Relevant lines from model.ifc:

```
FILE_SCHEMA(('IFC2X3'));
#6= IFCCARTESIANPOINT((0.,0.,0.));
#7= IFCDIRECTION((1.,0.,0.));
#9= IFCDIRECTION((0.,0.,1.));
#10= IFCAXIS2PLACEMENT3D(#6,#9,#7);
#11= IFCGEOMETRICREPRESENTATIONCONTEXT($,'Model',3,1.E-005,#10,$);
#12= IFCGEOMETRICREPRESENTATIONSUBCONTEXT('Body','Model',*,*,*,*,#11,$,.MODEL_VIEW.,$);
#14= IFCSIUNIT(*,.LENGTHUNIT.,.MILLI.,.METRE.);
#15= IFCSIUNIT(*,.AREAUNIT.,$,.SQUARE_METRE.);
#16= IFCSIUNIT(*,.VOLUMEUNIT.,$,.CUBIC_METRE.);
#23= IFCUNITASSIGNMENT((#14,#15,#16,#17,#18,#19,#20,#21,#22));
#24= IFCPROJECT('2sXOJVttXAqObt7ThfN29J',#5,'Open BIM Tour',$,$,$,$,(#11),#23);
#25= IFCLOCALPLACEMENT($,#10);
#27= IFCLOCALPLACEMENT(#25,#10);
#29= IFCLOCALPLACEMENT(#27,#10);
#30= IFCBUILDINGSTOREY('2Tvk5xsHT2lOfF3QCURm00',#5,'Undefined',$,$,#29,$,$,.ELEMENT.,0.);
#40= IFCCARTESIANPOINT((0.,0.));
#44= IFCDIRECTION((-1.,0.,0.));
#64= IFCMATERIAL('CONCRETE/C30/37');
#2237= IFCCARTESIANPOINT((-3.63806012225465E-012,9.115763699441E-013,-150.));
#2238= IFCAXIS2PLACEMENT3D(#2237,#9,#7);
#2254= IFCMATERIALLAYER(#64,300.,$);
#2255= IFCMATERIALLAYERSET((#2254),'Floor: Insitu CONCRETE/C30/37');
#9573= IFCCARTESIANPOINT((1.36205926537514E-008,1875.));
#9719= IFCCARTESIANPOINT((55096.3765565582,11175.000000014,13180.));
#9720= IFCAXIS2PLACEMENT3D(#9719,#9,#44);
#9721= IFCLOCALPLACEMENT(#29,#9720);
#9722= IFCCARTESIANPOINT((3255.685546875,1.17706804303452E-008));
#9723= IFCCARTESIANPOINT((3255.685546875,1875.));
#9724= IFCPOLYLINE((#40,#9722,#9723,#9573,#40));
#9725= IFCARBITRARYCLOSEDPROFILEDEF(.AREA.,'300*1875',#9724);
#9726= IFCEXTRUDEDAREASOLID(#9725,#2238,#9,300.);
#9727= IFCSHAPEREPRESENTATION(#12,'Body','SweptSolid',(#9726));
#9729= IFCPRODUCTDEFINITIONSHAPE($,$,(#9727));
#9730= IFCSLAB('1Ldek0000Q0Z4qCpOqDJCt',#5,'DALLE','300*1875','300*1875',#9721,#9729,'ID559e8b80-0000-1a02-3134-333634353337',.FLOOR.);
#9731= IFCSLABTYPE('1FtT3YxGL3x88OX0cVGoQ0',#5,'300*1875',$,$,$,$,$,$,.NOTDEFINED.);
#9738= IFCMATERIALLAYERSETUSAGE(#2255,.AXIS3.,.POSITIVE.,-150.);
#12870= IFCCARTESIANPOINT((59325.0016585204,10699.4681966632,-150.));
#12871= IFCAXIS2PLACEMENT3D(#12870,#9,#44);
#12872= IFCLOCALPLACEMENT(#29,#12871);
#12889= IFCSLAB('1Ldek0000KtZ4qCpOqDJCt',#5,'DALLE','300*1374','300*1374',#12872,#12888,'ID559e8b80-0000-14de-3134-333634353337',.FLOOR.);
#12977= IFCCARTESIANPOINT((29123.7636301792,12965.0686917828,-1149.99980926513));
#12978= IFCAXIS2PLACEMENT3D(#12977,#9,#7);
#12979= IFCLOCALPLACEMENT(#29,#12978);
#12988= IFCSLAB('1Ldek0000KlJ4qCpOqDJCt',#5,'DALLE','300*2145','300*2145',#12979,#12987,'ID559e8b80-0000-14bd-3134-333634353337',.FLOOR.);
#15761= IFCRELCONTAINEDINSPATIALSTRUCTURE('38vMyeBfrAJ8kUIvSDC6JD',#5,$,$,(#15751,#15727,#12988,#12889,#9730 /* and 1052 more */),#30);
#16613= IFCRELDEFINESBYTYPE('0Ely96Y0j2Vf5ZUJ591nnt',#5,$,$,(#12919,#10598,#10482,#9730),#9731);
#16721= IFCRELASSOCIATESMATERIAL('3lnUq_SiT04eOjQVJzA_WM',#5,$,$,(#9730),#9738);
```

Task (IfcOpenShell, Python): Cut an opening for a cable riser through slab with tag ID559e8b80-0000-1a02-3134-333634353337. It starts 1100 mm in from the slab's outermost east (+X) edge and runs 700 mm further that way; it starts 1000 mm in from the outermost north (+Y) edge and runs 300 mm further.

```python
import numpy as np
import ifcopenshell
import ifcopenshell.api.feature
import ifcopenshell.api.geometry
import ifcopenshell.api.root
import ifcopenshell.geom
import ifcopenshell.util.placement
import ifcopenshell.util.representation
import ifcopenshell.util.shape
import ifcopenshell.util.unit

model = ifcopenshell.open("model.ifc")
unit_scale = ifcopenshell.util.unit.calculate_unit_scale(model)
settings = ifcopenshell.geom.settings()


def volume(element):
    """Net volume in cubic metres, openings subtracted."""
    shape = ifcopenshell.geom.create_shape(settings, element)
    return ifcopenshell.util.shape.get_volume(shape.geometry)


slab = model.by_id(9730)
before = volume(slab)

# Extent in the slab's own axes, in metres. The edges named are its -X and -Y sides.
slab_shape = ifcopenshell.geom.create_shape(settings, slab)
vertices = ifcopenshell.util.shape.get_vertices(slab_shape.geometry)
x_min, y_min, bottom = vertices.min(axis=0)
top = vertices[:, 2].max()

opening = ifcopenshell.api.root.create_entity(model, ifc_class="IfcOpeningElement", name="Cable riser opening")
context = ifcopenshell.util.representation.get_context(model, "Model", "Body", "MODEL_VIEW")
width, depth = 0.7, 0.3
outline = [(0.0, 0.0), (width, 0.0), (width, depth), (0.0, depth), (0.0, 0.0)]
# Overshoot both faces by 50 mm so the cut is clean.
shape = ifcopenshell.api.geometry.add_slab_representation(
    model, context=context, depth=top - bottom + 0.1, polyline=outline
)
ifcopenshell.api.geometry.assign_representation(model, product=opening, representation=shape)

matrix = ifcopenshell.util.placement.get_local_placement(slab.ObjectPlacement)
matrix[:, 3] = matrix @ np.append(np.array([x_min + 1.1, y_min + 1, bottom - 0.05]) / unit_scale, 1.0)
ifcopenshell.api.geometry.edit_object_placement(model, product=opening, matrix=matrix, is_si=False)
ifcopenshell.api.feature.add_feature(model, feature=opening, element=slab)

after = volume(slab)

print(f"slab volume {before:.3f} -> {after:.3f} m3")

model.write("model_rev.ifc")
```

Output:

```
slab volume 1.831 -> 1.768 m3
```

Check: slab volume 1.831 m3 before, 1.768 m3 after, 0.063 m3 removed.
